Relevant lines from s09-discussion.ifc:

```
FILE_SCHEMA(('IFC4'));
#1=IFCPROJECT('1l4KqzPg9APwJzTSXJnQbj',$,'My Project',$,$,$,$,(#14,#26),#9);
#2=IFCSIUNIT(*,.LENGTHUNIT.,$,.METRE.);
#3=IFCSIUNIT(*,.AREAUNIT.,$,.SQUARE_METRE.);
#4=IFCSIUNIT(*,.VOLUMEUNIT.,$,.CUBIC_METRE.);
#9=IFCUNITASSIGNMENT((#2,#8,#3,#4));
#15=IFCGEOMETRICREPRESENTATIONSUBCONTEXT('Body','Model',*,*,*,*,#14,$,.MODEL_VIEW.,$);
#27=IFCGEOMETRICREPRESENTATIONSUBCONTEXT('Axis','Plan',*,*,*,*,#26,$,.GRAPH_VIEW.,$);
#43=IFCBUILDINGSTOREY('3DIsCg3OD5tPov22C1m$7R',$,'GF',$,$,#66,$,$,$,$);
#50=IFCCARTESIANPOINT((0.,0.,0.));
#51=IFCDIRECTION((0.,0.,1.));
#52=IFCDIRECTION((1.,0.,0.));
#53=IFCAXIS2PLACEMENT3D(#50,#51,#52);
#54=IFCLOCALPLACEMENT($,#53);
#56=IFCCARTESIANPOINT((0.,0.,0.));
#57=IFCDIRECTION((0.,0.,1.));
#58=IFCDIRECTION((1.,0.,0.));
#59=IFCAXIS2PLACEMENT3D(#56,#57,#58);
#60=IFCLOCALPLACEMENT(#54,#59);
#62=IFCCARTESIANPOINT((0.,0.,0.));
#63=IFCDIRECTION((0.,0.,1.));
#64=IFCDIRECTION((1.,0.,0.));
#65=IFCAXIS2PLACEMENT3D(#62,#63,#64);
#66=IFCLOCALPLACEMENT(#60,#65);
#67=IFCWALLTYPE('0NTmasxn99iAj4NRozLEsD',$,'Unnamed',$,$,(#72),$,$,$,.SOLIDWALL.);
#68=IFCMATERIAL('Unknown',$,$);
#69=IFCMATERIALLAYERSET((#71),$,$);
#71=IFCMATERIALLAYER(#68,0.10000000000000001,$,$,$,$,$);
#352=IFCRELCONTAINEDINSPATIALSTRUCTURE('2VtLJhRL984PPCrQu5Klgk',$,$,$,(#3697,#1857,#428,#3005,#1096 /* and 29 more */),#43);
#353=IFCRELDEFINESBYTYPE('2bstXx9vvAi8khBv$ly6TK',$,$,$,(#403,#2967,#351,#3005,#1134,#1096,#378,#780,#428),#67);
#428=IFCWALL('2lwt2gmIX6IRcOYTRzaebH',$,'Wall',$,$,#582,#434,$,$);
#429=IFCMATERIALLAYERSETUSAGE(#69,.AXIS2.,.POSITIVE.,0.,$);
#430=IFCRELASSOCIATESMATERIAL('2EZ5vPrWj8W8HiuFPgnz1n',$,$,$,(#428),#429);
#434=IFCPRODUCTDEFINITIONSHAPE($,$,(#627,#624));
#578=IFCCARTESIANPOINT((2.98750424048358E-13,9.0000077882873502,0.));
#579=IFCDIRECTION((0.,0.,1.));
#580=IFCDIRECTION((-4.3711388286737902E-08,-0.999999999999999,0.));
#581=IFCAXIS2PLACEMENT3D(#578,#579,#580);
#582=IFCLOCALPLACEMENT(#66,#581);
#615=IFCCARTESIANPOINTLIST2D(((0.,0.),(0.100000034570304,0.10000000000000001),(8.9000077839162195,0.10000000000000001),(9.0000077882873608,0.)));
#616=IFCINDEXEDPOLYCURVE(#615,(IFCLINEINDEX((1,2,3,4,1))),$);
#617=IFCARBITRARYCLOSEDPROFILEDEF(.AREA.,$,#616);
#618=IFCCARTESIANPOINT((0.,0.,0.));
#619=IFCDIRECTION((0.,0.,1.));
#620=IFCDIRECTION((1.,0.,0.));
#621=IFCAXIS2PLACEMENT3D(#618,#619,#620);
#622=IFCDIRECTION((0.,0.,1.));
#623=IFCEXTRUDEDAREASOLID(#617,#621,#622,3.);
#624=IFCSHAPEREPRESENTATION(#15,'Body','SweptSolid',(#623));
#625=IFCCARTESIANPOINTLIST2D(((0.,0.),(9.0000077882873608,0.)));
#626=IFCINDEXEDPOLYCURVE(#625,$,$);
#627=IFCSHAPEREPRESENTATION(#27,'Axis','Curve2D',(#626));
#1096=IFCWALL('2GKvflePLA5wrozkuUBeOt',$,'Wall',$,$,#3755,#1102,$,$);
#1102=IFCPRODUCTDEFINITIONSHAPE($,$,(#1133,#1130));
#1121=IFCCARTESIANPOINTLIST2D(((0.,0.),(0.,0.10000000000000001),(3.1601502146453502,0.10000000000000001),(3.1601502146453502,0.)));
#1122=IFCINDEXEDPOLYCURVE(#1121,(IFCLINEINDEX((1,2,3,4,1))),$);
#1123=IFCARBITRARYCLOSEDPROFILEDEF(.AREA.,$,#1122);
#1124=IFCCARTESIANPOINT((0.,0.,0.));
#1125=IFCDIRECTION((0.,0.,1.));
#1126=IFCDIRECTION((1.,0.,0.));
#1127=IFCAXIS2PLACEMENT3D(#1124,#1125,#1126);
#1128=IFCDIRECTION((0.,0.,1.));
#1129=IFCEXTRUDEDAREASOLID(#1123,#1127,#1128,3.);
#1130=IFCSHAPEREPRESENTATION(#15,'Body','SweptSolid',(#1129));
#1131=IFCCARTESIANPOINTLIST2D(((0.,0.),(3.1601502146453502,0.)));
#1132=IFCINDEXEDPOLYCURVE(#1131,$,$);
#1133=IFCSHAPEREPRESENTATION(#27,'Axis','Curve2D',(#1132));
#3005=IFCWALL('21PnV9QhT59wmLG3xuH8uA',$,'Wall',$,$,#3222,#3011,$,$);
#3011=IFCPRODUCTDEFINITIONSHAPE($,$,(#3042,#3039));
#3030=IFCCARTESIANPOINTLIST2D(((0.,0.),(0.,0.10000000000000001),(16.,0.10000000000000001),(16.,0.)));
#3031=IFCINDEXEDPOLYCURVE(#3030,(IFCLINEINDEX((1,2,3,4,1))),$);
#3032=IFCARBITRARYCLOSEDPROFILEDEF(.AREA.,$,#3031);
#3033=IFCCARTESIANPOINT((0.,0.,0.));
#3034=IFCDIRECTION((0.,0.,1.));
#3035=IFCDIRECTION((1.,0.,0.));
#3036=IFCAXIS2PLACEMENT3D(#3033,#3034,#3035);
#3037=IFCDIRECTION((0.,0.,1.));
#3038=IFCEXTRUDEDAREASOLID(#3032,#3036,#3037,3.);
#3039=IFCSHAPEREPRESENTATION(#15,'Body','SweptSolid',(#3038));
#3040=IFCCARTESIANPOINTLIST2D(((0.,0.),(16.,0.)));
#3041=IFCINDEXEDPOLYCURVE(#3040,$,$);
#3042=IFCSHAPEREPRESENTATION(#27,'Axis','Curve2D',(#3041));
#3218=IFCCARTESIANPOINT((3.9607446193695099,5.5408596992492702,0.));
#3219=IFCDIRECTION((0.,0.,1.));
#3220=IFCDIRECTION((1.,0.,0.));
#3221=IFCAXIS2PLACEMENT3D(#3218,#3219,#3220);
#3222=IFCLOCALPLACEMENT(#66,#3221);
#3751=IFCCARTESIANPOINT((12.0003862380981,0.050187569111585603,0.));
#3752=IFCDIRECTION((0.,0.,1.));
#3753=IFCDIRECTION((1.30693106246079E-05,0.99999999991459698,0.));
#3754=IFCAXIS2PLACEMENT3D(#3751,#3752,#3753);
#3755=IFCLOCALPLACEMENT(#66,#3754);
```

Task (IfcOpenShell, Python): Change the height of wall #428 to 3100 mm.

```python
import ifcopenshell
import ifcopenshell.geom
import ifcopenshell.util.representation
import ifcopenshell.util.shape
import ifcopenshell.util.unit

model = ifcopenshell.open("s09-discussion.ifc")
unit_scale = ifcopenshell.util.unit.calculate_unit_scale(model)
settings = ifcopenshell.geom.settings()


def volume(element):
    """Net volume in cubic metres, openings subtracted."""
    shape = ifcopenshell.geom.create_shape(settings, element)
    return ifcopenshell.util.shape.get_volume(shape.geometry)


wall = model.by_guid("2lwt2gmIX6IRcOYTRzaebH")
before = volume(wall)

body = ifcopenshell.util.representation.get_representation(wall, "Model", "Body")
solid = body.Items[0]
old_height = solid.Depth
solid.Depth = 3.1 / unit_scale
after = volume(wall)

print(f"height {old_height:g} -> {solid.Depth:g}, volume {before:.3f} -> {after:.3f} m3")

model.write("s09-discussion_rev.ifc")
```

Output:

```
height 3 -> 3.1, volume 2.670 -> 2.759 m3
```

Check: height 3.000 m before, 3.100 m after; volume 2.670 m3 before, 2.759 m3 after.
